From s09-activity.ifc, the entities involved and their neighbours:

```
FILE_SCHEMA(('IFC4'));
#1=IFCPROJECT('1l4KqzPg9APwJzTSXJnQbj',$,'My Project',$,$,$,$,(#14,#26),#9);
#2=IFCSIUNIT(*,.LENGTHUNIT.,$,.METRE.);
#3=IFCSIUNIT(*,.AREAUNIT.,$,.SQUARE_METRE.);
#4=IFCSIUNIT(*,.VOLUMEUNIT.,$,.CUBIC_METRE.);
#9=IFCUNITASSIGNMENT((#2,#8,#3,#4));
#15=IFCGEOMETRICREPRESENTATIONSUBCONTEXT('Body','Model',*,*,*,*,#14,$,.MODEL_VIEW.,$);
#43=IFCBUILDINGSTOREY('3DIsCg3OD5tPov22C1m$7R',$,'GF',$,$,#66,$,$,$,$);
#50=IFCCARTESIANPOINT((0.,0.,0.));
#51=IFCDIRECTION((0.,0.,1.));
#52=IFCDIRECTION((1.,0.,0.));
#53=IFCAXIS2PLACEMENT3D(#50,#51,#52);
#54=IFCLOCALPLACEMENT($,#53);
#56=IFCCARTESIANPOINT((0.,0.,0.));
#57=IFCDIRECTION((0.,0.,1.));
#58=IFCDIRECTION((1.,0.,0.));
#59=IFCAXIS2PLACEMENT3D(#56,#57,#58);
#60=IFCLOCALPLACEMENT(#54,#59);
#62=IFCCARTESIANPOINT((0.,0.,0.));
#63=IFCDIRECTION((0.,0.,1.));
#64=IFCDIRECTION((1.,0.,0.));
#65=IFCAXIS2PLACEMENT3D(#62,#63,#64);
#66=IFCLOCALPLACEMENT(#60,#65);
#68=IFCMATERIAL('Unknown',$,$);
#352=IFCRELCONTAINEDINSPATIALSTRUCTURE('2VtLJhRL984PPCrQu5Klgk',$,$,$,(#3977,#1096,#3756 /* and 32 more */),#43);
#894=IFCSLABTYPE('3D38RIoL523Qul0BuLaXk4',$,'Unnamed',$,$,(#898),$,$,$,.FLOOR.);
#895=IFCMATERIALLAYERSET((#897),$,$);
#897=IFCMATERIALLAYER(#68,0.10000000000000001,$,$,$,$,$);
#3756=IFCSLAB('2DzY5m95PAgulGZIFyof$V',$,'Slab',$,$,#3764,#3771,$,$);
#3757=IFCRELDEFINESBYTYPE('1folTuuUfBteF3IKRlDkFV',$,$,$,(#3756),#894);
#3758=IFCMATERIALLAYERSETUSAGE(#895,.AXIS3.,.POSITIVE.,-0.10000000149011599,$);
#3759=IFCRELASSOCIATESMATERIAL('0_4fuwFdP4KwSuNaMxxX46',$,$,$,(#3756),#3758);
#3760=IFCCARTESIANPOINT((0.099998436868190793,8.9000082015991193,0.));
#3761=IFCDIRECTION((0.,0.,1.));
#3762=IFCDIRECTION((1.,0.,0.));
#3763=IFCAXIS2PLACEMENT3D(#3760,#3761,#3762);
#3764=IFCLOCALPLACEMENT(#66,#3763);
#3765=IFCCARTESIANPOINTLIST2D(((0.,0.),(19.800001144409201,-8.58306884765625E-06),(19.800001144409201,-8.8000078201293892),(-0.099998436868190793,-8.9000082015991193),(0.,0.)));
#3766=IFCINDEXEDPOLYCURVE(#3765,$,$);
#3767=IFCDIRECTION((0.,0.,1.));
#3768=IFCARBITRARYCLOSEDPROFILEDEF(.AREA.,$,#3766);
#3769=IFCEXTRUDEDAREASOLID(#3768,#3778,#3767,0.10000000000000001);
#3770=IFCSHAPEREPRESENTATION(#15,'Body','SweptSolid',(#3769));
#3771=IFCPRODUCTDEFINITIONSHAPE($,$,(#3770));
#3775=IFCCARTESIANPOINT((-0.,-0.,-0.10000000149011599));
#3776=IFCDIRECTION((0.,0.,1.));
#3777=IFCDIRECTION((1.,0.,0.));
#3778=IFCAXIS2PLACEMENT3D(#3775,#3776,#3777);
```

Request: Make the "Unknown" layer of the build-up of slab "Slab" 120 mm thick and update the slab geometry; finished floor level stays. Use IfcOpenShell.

```python
import ifcopenshell
import ifcopenshell.util.element
import ifcopenshell.util.representation
import ifcopenshell.util.unit

model = ifcopenshell.open("s09-activity.ifc")
unit_scale = ifcopenshell.util.unit.calculate_unit_scale(model)

layer_set = model.by_id(895)
layer = next(l for l in layer_set.MaterialLayers if l.Material and l.Material.Name == "Unknown")
change = 0.12 / unit_scale - layer.LayerThickness
layer.LayerThickness += change

# Geometry does not follow the layer set by itself.
slabs = [e for e in ifcopenshell.util.element.get_elements_by_material(model, layer_set) if e.is_a("IfcSlab")]
for slab in sorted(slabs, key=lambda e: e.id()):
    body = ifcopenshell.util.representation.get_representation(slab, "Model", "Body")
    solid = body.Items[0]
    old_depth = solid.Depth
    solid.Depth += change
    # Extruded upwards: lower the start of the extrusion so the top stays.
    x, y, z = solid.Position.Location.Coordinates
    solid.Position.Location = model.createIfcCartesianPoint((x, y, z - change))
    print(slab.id(), f"{old_depth:g} -> {solid.Depth:g}")

# The layers are counted up from the underside, which has moved.
for usage in {ifcopenshell.util.element.get_material(slab) for slab in slabs}:
    usage.OffsetFromReferenceLine -= change

model.write("s09-activity_edited.ifc")
```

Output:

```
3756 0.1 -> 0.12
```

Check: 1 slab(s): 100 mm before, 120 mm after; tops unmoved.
